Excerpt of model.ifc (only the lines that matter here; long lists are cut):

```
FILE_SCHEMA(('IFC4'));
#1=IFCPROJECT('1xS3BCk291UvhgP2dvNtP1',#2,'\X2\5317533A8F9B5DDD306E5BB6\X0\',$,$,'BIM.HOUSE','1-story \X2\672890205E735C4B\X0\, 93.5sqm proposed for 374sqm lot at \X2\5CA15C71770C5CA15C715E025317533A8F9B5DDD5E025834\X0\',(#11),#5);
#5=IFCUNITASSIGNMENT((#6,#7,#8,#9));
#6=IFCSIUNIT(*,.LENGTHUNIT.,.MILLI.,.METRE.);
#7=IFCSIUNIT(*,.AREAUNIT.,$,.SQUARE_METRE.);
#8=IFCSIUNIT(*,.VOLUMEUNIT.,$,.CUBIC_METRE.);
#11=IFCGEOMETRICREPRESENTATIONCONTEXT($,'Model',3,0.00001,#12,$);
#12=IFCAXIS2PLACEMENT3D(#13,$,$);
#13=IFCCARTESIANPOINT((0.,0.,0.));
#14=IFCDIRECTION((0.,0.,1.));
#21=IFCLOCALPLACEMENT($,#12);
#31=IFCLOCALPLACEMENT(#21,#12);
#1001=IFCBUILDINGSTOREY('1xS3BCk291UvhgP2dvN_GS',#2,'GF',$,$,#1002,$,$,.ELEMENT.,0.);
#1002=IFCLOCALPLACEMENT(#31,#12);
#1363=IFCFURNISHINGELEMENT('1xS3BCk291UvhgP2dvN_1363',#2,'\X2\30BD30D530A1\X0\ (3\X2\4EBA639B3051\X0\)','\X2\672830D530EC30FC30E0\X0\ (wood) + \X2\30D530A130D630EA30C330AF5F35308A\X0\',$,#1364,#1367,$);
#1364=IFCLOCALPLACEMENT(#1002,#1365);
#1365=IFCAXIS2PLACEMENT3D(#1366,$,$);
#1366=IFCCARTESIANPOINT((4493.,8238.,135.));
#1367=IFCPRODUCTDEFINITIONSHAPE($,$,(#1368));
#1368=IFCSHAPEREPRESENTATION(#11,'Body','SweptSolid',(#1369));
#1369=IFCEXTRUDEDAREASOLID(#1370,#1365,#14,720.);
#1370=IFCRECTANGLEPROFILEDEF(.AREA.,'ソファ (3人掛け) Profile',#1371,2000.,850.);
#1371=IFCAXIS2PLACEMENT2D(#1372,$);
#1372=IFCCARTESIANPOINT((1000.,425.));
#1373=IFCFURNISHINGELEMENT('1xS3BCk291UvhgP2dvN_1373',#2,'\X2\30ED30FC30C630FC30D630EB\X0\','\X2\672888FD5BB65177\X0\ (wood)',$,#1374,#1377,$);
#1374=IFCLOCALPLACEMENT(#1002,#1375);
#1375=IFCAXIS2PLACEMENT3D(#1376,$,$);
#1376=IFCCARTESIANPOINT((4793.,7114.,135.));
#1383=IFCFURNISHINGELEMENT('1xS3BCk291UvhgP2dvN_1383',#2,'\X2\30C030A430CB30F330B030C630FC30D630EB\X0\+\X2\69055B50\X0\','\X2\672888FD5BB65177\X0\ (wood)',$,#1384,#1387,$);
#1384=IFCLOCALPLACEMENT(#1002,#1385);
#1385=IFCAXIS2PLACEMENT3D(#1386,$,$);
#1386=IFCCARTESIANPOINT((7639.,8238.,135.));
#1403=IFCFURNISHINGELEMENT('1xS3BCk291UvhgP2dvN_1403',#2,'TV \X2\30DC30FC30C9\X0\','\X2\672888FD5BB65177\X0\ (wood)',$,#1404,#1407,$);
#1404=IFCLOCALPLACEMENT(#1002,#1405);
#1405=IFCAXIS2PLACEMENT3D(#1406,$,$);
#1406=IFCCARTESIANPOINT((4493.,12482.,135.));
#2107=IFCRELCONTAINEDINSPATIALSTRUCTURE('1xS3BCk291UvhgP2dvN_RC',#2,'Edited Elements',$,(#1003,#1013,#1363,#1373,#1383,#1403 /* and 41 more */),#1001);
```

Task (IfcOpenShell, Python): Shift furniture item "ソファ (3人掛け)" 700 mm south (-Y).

```python
import ifcopenshell
import ifcopenshell.api.geometry
import ifcopenshell.util.placement
import ifcopenshell.util.unit

model = ifcopenshell.open("model.ifc")
unit_scale = ifcopenshell.util.unit.calculate_unit_scale(model)

item = model.by_guid("1xS3BCk291UvhgP2dvN_1363")
matrix = ifcopenshell.util.placement.get_local_placement(item.ObjectPlacement)
matrix[1, 3] -= 0.7 / unit_scale
ifcopenshell.api.geometry.edit_object_placement(model, product=item, matrix=matrix, is_si=False)

print(ifcopenshell.util.placement.get_local_placement(item.ObjectPlacement).round(3) + 0.0)

model.write("model_v2.ifc")
```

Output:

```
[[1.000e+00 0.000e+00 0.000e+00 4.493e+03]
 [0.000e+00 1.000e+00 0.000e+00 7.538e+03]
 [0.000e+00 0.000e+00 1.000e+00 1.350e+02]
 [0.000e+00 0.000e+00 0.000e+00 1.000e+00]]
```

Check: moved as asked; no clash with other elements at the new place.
